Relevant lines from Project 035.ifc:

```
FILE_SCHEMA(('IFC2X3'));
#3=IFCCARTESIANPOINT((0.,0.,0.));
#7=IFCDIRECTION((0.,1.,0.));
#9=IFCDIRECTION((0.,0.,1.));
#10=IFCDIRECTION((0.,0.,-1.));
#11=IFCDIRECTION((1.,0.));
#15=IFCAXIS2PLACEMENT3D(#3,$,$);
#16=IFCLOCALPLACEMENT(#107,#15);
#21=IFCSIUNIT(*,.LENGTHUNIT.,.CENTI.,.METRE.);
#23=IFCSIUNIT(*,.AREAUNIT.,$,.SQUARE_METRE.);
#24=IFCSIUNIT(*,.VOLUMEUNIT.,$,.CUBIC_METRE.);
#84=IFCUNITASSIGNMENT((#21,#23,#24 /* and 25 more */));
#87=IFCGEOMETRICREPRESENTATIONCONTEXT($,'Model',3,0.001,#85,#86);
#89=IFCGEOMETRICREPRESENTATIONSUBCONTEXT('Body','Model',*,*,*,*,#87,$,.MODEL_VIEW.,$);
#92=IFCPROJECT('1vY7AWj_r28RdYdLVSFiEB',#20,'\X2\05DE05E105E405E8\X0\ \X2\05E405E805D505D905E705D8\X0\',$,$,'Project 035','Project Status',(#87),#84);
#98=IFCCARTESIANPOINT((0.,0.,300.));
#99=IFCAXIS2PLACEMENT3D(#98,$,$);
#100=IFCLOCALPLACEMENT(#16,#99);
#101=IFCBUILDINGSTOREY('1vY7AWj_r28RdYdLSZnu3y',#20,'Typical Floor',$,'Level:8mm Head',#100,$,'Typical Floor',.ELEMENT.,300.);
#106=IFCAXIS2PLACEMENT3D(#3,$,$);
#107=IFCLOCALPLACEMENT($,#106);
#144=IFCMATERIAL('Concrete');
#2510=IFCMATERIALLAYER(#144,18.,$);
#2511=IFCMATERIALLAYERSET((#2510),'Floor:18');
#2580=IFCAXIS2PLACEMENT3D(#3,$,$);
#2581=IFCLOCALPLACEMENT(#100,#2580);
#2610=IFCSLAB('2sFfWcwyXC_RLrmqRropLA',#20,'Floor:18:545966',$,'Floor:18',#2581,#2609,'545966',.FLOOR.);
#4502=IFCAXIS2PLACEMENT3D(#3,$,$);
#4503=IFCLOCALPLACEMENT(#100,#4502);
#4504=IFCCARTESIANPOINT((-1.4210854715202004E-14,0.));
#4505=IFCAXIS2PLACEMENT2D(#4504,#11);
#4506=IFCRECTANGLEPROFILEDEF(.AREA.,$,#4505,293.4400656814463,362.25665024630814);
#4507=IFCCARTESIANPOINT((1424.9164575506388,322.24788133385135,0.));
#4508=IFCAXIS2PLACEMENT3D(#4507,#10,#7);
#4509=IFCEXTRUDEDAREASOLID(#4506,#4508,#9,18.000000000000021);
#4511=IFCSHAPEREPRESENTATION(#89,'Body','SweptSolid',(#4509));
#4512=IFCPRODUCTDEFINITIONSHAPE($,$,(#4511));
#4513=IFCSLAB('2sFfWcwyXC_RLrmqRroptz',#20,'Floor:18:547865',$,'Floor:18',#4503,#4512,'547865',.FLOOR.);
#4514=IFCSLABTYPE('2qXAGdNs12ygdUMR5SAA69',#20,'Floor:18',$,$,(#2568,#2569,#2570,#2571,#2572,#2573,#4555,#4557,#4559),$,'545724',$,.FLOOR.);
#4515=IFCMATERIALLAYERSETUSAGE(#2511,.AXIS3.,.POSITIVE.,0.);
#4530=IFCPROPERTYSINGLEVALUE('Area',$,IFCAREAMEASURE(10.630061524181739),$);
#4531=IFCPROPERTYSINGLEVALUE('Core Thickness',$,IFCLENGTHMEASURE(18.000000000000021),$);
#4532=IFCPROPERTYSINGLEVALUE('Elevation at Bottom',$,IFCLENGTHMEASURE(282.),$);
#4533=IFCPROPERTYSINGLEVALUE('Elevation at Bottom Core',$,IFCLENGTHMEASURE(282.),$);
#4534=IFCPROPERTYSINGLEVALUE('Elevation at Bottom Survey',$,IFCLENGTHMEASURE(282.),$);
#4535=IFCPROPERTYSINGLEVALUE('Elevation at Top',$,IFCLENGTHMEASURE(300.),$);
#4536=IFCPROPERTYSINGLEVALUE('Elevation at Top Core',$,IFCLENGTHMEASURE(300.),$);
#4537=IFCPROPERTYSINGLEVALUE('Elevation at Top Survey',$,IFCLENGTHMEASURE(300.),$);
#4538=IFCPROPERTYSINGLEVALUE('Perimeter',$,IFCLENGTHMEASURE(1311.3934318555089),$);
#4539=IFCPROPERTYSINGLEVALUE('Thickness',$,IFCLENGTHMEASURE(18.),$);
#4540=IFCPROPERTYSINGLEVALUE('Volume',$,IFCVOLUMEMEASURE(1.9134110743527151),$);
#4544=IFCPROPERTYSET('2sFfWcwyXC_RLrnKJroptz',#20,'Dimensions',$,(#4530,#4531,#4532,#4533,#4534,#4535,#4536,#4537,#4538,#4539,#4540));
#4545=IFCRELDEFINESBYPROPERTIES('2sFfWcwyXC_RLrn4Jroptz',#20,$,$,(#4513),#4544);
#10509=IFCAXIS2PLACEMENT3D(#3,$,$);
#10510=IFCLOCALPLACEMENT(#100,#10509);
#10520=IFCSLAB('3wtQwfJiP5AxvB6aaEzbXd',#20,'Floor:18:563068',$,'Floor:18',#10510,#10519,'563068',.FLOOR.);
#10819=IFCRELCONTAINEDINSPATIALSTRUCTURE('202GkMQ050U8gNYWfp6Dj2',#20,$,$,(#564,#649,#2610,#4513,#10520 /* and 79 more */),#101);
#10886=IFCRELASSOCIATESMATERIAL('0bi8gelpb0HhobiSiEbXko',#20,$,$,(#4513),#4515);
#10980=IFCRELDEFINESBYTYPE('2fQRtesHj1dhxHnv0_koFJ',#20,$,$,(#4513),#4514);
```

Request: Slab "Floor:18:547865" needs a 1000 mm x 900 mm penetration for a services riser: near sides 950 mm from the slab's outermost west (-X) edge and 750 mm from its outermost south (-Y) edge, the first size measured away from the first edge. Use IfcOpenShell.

```python
import numpy as np
import ifcopenshell
import ifcopenshell.api.feature
import ifcopenshell.api.geometry
import ifcopenshell.api.pset
import ifcopenshell.api.root
import ifcopenshell.geom
import ifcopenshell.util.element
import ifcopenshell.util.placement
import ifcopenshell.util.representation
import ifcopenshell.util.shape
import ifcopenshell.util.unit

model = ifcopenshell.open("Project 035.ifc")
unit_scale = ifcopenshell.util.unit.calculate_unit_scale(model)
area_scale = ifcopenshell.util.unit.calculate_unit_scale(model, "AREAUNIT")
volume_scale = ifcopenshell.util.unit.calculate_unit_scale(model, "VOLUMEUNIT")
settings = ifcopenshell.geom.settings()


def volume(element):
    """Net volume in cubic metres, openings subtracted."""
    shape = ifcopenshell.geom.create_shape(settings, element)
    return ifcopenshell.util.shape.get_volume(shape.geometry)


slab = model.by_guid("2sFfWcwyXC_RLrmqRroptz")
before = volume(slab)

# Extent in the slab's own axes, in metres. The edges named are its -X and -Y sides.
slab_shape = ifcopenshell.geom.create_shape(settings, slab)
vertices = ifcopenshell.util.shape.get_vertices(slab_shape.geometry)
x_min, y_min, bottom = vertices.min(axis=0)
top = vertices[:, 2].max()

opening = ifcopenshell.api.root.create_entity(model, ifc_class="IfcOpeningElement", name="Services riser opening")
context = ifcopenshell.util.representation.get_context(model, "Model", "Body", "MODEL_VIEW")
width, depth = 1, 0.9
outline = [(0.0, 0.0), (width, 0.0), (width, depth), (0.0, depth), (0.0, 0.0)]
# Overshoot both faces by 50 mm so the cut is clean.
shape = ifcopenshell.api.geometry.add_slab_representation(
    model, context=context, depth=top - bottom + 0.1, polyline=outline
)
ifcopenshell.api.geometry.assign_representation(model, product=opening, representation=shape)

matrix = ifcopenshell.util.placement.get_local_placement(slab.ObjectPlacement)
matrix[:, 3] = matrix @ np.append(np.array([x_min + 0.95, y_min + 0.75, bottom - 0.05]) / unit_scale, 1.0)
ifcopenshell.api.geometry.edit_object_placement(model, product=opening, matrix=matrix, is_si=False)
ifcopenshell.api.feature.add_feature(model, feature=opening, element=slab)

after = volume(slab)

# Update the slab's stored quantities.
pset = model.by_id(ifcopenshell.util.element.get_pset(slab, "Dimensions", should_inherit=False)["id"])
ifcopenshell.api.pset.edit_pset(model, pset=pset, properties={
    "Area": model.create_entity("IfcAreaMeasure", after / (top - bottom) / area_scale),
    "Volume": model.create_entity("IfcVolumeMeasure", after / volume_scale),
})

print(f"slab volume {before:.3f} -> {after:.3f} m3")

model.write("Project 035_updated.ifc")
```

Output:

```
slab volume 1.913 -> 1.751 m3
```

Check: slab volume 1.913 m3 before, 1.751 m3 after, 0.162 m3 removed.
